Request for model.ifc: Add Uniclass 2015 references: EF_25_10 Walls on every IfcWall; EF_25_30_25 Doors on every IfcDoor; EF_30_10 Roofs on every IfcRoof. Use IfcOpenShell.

First a look at what the model holds.

```python
import ifcopenshell

model = ifcopenshell.open("model.ifc")
print(model.schema)
print("classifications:", [c.Name for c in model.by_type("IfcClassification")])
for ifc_class in ("IfcDoor", "IfcRoof", "IfcStair", "IfcWall", "IfcWindow"):
    print(ifc_class, len(model.by_type(ifc_class)))
```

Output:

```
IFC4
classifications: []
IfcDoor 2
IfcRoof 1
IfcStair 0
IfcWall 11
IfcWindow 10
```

```python
import ifcopenshell
import ifcopenshell.api.classification

model = ifcopenshell.open("model.ifc")

system = ifcopenshell.api.classification.add_classification(model, classification="Uniclass 2015")

codes = {
    "IfcWall": ("EF_25_10", "Walls"),
    "IfcDoor": ("EF_25_30_25", "Doors"),
    "IfcRoof": ("EF_30_10", "Roofs"),
}
for ifc_class, (code, name) in codes.items():
    products = model.by_type(ifc_class)
    ifcopenshell.api.classification.add_reference(
        model, products=products, classification=system, identification=code, name=name
    )
    print(code, len(products))

model.write("model_updated.ifc")
```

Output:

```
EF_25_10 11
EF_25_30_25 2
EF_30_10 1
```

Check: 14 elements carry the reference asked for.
